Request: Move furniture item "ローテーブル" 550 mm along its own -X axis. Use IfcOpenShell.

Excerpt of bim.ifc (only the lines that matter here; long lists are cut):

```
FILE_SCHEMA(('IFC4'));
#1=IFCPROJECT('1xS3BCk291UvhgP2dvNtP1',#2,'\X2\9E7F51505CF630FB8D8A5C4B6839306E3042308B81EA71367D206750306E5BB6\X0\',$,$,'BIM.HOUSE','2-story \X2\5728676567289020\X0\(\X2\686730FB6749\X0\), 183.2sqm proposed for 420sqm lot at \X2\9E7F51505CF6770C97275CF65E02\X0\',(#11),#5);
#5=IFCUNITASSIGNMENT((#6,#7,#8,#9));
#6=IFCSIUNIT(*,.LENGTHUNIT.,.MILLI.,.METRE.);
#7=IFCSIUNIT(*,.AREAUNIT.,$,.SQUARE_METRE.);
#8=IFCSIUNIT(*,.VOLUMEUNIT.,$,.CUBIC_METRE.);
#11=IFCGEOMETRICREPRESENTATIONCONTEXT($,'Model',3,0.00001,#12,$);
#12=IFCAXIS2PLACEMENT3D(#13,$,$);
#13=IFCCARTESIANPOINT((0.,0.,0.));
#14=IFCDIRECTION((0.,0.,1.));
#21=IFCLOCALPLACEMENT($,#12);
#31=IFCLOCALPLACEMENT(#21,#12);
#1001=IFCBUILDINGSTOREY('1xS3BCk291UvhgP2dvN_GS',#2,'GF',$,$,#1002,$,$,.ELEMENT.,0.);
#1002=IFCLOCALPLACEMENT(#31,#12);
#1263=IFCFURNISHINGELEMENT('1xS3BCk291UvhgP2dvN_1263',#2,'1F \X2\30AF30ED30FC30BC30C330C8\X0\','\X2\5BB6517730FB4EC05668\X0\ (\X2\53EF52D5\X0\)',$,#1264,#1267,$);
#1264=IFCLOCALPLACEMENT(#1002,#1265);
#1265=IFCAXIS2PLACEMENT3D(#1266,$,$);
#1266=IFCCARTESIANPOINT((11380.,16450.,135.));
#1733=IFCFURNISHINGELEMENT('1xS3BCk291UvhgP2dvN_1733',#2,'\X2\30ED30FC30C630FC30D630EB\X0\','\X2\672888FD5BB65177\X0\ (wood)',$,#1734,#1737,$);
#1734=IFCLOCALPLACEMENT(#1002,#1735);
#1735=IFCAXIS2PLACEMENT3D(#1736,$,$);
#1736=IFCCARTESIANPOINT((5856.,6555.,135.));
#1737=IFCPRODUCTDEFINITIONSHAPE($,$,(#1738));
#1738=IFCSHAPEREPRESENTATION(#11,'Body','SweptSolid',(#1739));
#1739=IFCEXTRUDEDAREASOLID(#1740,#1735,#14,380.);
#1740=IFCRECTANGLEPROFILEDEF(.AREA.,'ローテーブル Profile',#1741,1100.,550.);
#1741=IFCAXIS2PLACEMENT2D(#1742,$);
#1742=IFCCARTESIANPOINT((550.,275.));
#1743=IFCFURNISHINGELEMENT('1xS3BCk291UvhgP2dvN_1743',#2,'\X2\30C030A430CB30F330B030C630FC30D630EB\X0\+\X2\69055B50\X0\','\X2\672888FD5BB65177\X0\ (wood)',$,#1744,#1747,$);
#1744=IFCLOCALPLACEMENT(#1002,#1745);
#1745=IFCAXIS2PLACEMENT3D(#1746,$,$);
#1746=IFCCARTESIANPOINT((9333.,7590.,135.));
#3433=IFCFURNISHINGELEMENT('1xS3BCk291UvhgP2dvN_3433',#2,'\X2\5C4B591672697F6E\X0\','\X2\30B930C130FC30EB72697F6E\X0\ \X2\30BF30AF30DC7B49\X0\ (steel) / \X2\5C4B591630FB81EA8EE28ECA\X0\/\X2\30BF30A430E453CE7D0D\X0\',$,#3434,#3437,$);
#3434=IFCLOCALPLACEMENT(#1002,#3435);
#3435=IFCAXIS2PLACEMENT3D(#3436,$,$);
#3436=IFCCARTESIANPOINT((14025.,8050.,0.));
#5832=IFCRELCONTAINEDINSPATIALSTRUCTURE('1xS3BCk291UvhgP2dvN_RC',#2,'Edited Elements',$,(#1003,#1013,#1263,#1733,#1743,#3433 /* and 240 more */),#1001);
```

```python
import ifcopenshell
import ifcopenshell.api.geometry
import ifcopenshell.util.placement
import ifcopenshell.util.unit

model = ifcopenshell.open("bim.ifc")
unit_scale = ifcopenshell.util.unit.calculate_unit_scale(model)

item = model.by_id(1733)
matrix = ifcopenshell.util.placement.get_local_placement(item.ObjectPlacement)
matrix[:3, 3] -= matrix[:3, 0] * 0.55 / unit_scale
ifcopenshell.api.geometry.edit_object_placement(model, product=item, matrix=matrix, is_si=False)

print(ifcopenshell.util.placement.get_local_placement(item.ObjectPlacement).round(3) + 0.0)

model.write("bim_updated.ifc")
```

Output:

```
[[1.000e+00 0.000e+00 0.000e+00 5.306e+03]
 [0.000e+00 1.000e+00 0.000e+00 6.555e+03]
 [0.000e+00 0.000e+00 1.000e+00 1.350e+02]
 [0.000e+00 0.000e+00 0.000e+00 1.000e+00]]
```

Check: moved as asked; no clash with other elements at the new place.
